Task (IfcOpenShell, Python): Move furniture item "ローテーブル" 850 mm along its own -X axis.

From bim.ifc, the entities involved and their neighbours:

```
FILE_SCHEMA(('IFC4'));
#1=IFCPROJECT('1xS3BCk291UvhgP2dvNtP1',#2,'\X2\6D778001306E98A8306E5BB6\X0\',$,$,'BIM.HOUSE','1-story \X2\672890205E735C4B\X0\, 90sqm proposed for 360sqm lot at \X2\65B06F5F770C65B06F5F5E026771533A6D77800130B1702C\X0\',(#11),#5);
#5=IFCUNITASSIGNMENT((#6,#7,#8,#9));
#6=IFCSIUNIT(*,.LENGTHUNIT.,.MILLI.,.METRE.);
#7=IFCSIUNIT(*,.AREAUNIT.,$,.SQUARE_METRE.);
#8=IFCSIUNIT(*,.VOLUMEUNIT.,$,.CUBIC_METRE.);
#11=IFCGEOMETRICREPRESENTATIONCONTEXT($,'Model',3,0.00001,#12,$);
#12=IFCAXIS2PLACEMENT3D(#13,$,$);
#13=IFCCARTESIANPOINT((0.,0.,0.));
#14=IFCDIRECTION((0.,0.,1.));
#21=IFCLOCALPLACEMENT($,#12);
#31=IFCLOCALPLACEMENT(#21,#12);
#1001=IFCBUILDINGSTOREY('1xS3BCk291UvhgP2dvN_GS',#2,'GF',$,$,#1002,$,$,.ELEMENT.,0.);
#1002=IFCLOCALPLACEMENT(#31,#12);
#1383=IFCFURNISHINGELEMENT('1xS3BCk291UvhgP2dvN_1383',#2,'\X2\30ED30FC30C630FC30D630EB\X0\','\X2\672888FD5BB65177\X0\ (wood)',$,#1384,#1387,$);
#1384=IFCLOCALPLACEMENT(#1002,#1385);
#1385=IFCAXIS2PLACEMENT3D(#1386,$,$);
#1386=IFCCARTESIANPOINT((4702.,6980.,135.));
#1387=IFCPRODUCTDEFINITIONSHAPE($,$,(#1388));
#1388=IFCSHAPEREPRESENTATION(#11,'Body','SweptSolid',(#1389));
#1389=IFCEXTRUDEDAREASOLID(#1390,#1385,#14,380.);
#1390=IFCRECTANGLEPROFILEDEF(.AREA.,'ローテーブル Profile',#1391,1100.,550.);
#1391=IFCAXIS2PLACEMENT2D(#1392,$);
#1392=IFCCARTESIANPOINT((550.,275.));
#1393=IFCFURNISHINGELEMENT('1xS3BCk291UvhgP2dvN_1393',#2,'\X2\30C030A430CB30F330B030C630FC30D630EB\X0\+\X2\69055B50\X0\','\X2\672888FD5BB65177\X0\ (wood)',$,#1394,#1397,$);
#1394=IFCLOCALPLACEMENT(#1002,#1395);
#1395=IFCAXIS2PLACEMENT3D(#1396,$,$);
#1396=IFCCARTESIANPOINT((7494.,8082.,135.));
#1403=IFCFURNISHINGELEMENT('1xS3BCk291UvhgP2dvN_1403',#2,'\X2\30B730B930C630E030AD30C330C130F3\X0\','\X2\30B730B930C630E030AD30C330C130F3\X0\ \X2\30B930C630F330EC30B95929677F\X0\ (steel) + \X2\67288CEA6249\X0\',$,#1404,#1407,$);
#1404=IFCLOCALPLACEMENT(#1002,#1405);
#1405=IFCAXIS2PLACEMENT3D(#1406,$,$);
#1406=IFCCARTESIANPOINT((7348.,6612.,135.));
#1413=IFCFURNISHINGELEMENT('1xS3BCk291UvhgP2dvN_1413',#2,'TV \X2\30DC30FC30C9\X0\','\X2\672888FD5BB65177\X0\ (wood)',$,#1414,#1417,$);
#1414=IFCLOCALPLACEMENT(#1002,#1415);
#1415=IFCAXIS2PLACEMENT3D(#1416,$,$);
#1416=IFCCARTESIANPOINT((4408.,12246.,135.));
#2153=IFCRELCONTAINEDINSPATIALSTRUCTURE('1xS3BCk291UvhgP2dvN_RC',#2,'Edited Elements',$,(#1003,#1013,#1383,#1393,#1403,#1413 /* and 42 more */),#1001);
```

```python
import ifcopenshell
import ifcopenshell.api.geometry
import ifcopenshell.util.placement
import ifcopenshell.util.unit

model = ifcopenshell.open("bim.ifc")
unit_scale = ifcopenshell.util.unit.calculate_unit_scale(model)

item = model.by_guid("1xS3BCk291UvhgP2dvN_1383")
matrix = ifcopenshell.util.placement.get_local_placement(item.ObjectPlacement)
matrix[:3, 3] -= matrix[:3, 0] * 0.85 / unit_scale
ifcopenshell.api.geometry.edit_object_placement(model, product=item, matrix=matrix, is_si=False)

print(ifcopenshell.util.placement.get_local_placement(item.ObjectPlacement).round(3) + 0.0)

model.write("bim_rev.ifc")
```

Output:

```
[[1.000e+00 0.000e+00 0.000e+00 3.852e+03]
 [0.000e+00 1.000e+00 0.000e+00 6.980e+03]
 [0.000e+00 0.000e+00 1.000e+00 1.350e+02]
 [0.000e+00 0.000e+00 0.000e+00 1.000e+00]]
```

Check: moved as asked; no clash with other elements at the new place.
